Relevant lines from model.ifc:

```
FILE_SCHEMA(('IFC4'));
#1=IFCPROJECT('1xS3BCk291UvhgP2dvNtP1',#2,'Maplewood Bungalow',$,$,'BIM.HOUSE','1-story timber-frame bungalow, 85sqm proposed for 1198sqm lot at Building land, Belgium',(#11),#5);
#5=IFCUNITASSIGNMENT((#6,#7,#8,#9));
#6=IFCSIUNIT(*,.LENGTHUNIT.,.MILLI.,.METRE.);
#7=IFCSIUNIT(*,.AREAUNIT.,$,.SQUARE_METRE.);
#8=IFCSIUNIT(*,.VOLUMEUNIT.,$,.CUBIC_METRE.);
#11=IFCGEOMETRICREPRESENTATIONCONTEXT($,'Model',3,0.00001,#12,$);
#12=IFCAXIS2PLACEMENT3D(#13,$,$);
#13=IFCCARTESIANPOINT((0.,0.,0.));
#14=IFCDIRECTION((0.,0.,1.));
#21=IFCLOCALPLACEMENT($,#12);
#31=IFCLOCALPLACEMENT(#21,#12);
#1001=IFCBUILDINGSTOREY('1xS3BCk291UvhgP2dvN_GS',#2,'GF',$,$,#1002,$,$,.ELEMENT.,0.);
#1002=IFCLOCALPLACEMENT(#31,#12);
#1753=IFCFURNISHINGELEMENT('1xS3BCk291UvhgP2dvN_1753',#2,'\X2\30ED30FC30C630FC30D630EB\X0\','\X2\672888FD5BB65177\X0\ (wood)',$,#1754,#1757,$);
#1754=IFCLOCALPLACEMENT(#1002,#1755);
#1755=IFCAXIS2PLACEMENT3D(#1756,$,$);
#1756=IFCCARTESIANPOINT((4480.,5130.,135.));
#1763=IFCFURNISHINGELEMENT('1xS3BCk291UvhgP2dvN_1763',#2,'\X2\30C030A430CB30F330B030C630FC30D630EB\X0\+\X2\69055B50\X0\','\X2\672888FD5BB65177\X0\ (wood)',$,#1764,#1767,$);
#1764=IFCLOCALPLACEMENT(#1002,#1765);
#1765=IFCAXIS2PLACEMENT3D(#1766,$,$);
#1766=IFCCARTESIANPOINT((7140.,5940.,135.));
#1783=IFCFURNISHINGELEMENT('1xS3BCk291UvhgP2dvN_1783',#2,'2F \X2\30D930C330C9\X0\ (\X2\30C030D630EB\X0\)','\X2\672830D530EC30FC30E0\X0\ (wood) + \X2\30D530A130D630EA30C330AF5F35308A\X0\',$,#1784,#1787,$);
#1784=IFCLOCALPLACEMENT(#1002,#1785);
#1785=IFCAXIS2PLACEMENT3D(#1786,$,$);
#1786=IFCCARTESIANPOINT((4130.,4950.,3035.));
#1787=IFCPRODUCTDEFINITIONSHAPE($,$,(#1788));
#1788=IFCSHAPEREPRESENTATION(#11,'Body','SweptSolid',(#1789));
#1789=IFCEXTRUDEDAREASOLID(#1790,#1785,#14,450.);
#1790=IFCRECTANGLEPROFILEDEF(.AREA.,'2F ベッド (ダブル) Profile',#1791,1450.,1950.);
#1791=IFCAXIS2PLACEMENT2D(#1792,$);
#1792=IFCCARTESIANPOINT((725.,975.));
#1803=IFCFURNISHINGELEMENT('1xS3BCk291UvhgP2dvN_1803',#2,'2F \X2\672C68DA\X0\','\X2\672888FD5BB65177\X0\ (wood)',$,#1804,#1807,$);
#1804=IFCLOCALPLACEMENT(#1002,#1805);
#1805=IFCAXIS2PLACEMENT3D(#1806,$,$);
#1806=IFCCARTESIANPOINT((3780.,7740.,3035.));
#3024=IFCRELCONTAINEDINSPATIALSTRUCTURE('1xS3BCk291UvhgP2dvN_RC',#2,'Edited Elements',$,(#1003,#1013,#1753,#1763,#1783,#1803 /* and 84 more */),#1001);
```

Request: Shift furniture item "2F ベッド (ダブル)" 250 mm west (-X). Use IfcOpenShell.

```python
import ifcopenshell
import ifcopenshell.api.geometry
import ifcopenshell.util.placement
import ifcopenshell.util.unit

model = ifcopenshell.open("model.ifc")
unit_scale = ifcopenshell.util.unit.calculate_unit_scale(model)

item = model.by_guid("1xS3BCk291UvhgP2dvN_1783")
matrix = ifcopenshell.util.placement.get_local_placement(item.ObjectPlacement)
matrix[0, 3] -= 0.25 / unit_scale
ifcopenshell.api.geometry.edit_object_placement(model, product=item, matrix=matrix, is_si=False)

print(ifcopenshell.util.placement.get_local_placement(item.ObjectPlacement).round(3) + 0.0)

model.write("model_edited.ifc")
```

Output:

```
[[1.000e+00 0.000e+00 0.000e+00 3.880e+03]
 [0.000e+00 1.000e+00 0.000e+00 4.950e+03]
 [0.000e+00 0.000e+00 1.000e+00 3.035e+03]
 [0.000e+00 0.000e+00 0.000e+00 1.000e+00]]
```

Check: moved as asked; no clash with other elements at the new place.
